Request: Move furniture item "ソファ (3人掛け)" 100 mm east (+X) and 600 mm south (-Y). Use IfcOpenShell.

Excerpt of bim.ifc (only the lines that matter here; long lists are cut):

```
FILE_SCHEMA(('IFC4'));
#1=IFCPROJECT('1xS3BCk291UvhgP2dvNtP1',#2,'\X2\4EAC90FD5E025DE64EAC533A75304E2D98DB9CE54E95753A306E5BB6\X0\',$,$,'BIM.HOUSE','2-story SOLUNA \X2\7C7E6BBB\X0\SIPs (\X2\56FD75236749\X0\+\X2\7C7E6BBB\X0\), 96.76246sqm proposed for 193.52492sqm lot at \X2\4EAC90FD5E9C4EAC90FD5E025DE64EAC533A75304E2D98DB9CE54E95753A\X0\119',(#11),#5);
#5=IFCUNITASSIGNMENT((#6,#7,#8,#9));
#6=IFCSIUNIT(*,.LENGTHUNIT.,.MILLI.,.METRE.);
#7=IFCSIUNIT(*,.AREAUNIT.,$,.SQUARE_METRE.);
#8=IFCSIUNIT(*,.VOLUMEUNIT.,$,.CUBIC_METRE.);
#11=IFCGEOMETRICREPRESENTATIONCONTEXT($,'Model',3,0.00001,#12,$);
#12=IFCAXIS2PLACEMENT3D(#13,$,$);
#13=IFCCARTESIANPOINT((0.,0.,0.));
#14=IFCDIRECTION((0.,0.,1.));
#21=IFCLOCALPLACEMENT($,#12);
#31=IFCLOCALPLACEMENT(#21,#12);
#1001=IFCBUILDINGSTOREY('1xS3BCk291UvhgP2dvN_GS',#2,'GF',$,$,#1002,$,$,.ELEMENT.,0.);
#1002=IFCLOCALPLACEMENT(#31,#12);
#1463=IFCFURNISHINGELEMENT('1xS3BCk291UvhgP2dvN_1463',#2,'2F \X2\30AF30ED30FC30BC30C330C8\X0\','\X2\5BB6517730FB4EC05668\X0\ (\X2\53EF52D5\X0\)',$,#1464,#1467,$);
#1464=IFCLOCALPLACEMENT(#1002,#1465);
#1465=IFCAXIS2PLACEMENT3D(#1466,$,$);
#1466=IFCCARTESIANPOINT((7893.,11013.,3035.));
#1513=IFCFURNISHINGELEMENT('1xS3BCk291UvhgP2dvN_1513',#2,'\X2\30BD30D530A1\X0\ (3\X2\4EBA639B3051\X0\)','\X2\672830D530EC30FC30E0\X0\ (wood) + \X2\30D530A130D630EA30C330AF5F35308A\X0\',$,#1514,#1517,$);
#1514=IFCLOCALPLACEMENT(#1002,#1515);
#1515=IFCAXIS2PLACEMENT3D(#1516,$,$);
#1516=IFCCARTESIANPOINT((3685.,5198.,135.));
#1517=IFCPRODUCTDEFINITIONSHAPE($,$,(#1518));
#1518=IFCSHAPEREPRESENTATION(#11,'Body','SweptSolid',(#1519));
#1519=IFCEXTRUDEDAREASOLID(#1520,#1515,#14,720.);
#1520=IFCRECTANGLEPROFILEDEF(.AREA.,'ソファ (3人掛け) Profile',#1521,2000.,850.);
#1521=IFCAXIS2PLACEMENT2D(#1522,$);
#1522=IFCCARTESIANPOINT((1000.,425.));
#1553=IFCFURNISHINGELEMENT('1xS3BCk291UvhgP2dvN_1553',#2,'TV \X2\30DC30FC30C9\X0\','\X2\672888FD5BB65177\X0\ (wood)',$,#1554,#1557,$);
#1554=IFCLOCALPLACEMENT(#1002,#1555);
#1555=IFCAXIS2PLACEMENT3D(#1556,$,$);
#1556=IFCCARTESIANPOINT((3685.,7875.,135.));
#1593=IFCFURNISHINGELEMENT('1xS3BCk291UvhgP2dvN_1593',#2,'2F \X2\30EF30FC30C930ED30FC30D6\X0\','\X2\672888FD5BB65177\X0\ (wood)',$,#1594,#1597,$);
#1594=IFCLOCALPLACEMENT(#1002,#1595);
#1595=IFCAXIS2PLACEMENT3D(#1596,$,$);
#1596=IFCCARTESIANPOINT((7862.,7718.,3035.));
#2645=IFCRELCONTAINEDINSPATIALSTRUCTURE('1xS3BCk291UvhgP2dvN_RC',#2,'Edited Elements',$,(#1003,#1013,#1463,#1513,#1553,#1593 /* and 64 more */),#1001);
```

```python
import ifcopenshell
import ifcopenshell.api.geometry
import ifcopenshell.util.placement
import ifcopenshell.util.unit

model = ifcopenshell.open("bim.ifc")
unit_scale = ifcopenshell.util.unit.calculate_unit_scale(model)

item = model.by_guid("1xS3BCk291UvhgP2dvN_1513")
matrix = ifcopenshell.util.placement.get_local_placement(item.ObjectPlacement)
matrix[0, 3] += 0.1 / unit_scale
matrix[1, 3] -= 0.6 / unit_scale
ifcopenshell.api.geometry.edit_object_placement(model, product=item, matrix=matrix, is_si=False)

print(ifcopenshell.util.placement.get_local_placement(item.ObjectPlacement).round(3) + 0.0)

model.write("bim_v2.ifc")
```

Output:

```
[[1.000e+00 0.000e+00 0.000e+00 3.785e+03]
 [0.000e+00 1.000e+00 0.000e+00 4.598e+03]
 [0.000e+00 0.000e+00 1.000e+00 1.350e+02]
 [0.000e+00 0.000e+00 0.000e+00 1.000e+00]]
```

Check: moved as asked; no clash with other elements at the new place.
